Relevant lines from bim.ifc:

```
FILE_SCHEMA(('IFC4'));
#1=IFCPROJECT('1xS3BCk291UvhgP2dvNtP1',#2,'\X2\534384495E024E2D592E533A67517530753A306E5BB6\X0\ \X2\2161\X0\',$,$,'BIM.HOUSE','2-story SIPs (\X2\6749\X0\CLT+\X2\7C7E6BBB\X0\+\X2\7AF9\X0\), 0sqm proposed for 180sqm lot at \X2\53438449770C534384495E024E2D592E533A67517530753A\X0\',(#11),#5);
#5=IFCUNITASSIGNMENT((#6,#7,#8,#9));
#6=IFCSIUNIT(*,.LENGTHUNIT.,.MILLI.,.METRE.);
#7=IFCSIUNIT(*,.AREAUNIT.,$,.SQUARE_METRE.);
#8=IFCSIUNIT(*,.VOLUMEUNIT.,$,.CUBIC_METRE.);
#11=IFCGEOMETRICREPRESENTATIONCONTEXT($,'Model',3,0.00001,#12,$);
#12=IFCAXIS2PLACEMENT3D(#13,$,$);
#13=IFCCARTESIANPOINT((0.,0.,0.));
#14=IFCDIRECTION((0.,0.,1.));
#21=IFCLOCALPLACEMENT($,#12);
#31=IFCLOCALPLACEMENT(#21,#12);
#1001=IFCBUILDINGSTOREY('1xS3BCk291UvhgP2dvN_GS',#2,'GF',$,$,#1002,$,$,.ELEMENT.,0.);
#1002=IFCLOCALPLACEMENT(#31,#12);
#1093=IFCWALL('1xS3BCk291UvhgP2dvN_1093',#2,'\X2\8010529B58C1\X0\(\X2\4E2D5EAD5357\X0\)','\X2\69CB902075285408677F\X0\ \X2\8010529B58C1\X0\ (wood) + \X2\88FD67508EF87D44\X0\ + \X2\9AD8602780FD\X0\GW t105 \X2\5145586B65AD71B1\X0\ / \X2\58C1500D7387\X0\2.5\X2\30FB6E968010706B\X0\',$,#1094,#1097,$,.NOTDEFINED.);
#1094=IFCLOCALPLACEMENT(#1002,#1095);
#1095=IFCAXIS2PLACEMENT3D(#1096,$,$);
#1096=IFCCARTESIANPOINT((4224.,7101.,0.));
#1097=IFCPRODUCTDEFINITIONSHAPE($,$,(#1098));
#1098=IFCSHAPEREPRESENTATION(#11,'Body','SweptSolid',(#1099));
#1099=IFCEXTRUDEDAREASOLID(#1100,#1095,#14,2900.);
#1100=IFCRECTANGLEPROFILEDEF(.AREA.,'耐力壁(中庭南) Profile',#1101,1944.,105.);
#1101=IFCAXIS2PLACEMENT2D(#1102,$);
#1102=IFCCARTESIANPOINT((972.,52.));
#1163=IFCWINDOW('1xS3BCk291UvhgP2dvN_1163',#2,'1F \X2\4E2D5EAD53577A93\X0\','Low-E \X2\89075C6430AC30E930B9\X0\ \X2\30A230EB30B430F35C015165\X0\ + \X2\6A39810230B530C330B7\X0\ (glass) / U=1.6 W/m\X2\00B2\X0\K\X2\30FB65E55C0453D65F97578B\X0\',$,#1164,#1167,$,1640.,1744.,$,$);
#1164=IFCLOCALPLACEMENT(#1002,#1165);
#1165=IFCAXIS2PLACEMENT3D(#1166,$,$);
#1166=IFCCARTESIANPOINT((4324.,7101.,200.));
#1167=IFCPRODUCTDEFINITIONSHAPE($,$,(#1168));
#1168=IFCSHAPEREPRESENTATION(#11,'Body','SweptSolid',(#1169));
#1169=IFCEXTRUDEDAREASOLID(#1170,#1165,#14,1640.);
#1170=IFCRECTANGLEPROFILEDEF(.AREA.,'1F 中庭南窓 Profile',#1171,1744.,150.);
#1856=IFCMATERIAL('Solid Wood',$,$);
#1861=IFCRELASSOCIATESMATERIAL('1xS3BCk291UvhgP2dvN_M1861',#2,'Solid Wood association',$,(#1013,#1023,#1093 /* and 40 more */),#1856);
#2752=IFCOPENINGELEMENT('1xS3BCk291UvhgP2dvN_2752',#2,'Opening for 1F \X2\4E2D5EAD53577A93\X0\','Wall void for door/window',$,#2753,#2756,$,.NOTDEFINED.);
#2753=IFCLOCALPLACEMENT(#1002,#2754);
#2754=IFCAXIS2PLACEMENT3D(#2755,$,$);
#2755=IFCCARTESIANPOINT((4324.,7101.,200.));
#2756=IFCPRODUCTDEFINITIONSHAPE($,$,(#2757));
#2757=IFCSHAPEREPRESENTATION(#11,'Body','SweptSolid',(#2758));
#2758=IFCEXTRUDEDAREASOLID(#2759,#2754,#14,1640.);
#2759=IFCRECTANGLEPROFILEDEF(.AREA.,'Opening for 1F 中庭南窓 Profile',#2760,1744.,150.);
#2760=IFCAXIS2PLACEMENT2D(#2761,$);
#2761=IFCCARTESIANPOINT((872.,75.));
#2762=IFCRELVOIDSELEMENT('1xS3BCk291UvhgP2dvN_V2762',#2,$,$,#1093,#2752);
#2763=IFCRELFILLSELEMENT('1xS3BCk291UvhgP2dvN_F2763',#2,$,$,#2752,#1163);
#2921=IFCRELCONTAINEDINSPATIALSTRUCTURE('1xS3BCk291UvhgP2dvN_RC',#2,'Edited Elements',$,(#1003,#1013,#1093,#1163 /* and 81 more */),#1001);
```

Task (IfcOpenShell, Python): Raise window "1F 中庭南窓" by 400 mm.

```python
import numpy as np
import ifcopenshell
import ifcopenshell.api.geometry
import ifcopenshell.util.placement
import ifcopenshell.util.unit

model = ifcopenshell.open("bim.ifc")
unit_scale = ifcopenshell.util.unit.calculate_unit_scale(model)

window = model.by_guid("1xS3BCk291UvhgP2dvN_1163")
opening = window.FillsVoids[0].RelatingOpeningElement
dz = 0.4 / unit_scale

shift = np.array([0.0, 0.0, dz])
# The window is not placed relative to its opening, so move both.
for product in (opening, window):
    matrix = ifcopenshell.util.placement.get_local_placement(product.ObjectPlacement)
    matrix[:3, 3] += shift
    ifcopenshell.api.geometry.edit_object_placement(model, product=product, matrix=matrix, is_si=False)

print(f"moved by {dz * unit_scale:+.3f} m")

model.write("bim-out.ifc")
```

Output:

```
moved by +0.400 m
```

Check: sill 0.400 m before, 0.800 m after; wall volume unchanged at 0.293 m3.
